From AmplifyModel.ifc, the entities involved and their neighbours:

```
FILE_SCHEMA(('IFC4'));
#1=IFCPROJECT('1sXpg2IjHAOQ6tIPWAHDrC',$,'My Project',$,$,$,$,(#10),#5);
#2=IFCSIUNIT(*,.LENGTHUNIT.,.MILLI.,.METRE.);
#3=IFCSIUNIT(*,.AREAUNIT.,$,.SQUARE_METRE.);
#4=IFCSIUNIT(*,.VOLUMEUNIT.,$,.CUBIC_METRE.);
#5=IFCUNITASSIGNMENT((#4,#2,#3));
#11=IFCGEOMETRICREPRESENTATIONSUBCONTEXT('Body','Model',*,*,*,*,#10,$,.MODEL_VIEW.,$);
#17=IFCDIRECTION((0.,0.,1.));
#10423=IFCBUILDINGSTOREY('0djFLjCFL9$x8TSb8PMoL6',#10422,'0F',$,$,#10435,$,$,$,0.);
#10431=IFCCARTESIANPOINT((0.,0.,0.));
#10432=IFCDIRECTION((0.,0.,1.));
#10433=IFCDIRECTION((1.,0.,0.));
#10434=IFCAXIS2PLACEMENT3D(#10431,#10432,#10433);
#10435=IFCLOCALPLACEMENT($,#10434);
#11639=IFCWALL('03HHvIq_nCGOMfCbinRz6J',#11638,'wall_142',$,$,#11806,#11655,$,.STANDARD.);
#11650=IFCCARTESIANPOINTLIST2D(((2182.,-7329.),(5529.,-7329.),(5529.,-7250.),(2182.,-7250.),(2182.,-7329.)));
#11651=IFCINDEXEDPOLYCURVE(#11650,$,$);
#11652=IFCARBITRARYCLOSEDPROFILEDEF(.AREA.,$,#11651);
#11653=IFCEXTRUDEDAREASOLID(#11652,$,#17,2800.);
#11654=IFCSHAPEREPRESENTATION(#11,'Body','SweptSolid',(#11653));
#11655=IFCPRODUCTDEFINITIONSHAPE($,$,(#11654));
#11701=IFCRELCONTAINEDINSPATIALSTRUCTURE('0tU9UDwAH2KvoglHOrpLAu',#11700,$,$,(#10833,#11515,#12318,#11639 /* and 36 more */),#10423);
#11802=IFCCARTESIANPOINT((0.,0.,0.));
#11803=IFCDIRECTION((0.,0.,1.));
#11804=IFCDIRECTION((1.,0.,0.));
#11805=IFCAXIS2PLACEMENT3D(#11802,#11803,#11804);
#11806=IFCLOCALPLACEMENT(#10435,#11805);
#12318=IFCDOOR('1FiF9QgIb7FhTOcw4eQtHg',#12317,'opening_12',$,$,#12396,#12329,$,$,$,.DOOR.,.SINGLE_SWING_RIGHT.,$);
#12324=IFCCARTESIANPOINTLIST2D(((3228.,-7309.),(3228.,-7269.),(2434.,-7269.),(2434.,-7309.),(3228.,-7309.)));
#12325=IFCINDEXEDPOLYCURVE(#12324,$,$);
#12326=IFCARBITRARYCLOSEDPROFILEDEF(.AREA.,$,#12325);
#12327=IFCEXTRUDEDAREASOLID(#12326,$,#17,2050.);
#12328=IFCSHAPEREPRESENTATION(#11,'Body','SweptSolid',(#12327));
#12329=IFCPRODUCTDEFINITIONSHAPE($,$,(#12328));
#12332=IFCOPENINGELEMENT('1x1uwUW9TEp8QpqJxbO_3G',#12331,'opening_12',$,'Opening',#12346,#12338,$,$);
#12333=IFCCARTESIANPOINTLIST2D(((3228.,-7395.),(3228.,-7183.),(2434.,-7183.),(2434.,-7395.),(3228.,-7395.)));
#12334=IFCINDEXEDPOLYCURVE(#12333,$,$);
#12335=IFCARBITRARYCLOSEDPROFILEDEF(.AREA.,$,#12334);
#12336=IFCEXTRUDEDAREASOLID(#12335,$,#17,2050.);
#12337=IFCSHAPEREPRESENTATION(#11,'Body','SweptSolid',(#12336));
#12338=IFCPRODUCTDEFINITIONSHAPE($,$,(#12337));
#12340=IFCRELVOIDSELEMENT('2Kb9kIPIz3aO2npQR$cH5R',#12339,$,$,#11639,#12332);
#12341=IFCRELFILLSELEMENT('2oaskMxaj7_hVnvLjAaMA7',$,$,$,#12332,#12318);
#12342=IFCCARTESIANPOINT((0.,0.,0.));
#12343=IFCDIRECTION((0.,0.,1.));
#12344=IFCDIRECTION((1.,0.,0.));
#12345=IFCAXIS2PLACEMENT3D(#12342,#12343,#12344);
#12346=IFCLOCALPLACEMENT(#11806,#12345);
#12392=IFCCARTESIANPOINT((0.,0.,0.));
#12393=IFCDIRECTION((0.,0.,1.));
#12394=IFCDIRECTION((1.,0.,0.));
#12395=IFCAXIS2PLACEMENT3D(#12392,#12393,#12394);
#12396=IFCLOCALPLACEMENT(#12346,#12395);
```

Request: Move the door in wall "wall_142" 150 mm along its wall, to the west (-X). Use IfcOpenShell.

```python
import ifcopenshell
import ifcopenshell.api.geometry
import ifcopenshell.util.placement

model = ifcopenshell.open("AmplifyModel.ifc")

door = model.by_guid("1FiF9QgIb7FhTOcw4eQtHg")
opening = door.FillsVoids[0].RelatingOpeningElement
wall = opening.VoidsElements[0].RelatingBuildingElement

wall_matrix = ifcopenshell.util.placement.get_local_placement(wall.ObjectPlacement)
shift = wall_matrix[:3, 0] * -150.0
before = ifcopenshell.util.placement.get_local_placement(door.ObjectPlacement)[:3, 3].copy()

# The door is placed relative to its opening, so it follows when the opening moves.
matrix = ifcopenshell.util.placement.get_local_placement(opening.ObjectPlacement)
matrix[:3, 3] += shift
ifcopenshell.api.geometry.edit_object_placement(
    model, product=opening, matrix=matrix, is_si=False, should_transform_children=True
)

after = ifcopenshell.util.placement.get_local_placement(door.ObjectPlacement)[:3, 3]
print("door moved by", (after - before).round(3) + 0.0)

model.write("AmplifyModel_updated.ifc")
```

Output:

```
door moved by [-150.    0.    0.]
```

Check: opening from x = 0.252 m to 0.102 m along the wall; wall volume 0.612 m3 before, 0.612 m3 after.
